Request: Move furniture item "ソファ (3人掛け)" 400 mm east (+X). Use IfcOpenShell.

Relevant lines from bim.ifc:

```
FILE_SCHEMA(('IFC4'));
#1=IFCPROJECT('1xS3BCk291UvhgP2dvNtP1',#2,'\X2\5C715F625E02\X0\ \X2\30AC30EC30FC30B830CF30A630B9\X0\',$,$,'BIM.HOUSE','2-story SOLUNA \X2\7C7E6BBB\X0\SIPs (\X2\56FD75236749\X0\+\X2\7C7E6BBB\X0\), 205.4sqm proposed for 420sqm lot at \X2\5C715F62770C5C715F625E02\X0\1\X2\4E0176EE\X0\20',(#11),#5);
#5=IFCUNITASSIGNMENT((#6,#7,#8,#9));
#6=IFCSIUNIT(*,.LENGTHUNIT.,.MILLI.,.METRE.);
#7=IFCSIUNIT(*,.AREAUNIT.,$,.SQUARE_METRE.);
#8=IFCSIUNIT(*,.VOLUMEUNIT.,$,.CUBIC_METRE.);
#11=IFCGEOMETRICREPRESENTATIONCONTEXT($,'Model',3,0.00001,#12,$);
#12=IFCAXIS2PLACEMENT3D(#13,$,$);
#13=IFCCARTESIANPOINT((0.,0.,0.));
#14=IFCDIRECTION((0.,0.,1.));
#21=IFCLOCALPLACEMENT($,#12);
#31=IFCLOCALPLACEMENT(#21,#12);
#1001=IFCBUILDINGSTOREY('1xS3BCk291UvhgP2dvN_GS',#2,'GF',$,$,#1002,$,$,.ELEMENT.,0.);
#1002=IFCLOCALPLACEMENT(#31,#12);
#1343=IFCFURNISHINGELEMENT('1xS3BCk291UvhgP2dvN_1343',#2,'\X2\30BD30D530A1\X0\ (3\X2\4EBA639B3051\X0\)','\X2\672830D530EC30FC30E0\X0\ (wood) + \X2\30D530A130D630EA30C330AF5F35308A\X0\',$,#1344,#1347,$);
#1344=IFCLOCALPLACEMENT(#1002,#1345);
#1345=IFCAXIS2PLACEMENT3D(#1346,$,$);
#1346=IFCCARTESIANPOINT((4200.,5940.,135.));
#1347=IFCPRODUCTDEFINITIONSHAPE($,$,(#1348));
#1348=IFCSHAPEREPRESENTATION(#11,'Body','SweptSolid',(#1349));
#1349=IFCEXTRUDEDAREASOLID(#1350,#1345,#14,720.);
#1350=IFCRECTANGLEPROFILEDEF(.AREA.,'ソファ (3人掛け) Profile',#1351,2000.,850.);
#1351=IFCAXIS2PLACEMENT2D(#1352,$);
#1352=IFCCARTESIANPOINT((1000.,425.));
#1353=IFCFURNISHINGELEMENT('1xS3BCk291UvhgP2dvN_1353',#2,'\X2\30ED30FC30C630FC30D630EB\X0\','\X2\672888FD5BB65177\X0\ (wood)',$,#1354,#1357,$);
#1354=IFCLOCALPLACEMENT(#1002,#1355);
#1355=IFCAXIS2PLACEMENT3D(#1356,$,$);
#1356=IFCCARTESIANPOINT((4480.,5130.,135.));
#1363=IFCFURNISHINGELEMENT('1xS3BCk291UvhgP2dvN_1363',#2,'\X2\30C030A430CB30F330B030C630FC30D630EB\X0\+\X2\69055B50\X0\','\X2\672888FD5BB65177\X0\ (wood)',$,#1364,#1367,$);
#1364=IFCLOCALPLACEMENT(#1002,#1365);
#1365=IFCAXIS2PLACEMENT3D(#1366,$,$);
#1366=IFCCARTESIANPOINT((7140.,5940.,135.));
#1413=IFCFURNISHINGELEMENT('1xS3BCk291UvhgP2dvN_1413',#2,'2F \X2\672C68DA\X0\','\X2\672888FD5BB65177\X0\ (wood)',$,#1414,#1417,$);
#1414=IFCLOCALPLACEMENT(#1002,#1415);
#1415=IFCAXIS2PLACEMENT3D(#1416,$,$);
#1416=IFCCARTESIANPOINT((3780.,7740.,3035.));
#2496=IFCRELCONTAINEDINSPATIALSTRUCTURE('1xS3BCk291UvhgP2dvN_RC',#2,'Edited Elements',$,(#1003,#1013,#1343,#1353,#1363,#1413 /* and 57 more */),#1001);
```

```python
import ifcopenshell
import ifcopenshell.api.geometry
import ifcopenshell.util.placement
import ifcopenshell.util.unit

model = ifcopenshell.open("bim.ifc")
unit_scale = ifcopenshell.util.unit.calculate_unit_scale(model)

item = model.by_guid("1xS3BCk291UvhgP2dvN_1343")
matrix = ifcopenshell.util.placement.get_local_placement(item.ObjectPlacement)
matrix[0, 3] += 0.4 / unit_scale
ifcopenshell.api.geometry.edit_object_placement(model, product=item, matrix=matrix, is_si=False)

print(ifcopenshell.util.placement.get_local_placement(item.ObjectPlacement).round(3) + 0.0)

model.write("bim_v2.ifc")
```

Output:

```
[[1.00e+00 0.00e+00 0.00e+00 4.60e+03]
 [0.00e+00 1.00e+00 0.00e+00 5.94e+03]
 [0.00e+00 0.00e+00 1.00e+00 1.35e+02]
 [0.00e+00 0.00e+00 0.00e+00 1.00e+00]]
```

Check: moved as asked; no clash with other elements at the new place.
